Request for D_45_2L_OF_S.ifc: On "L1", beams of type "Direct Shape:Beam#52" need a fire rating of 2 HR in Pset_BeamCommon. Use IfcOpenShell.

First a look at what the model holds.

```python
import ifcopenshell
import ifcopenshell.util.element

model = ifcopenshell.open("D_45_2L_OF_S.ifc")
print(model.schema)
storey = next(s for s in model.by_type("IfcBuildingStorey") if s.Name == "L1")
beams = [e for e in ifcopenshell.util.element.get_decomposition(storey) if e.is_a("IfcBeam")]
seen = {}
for e in beams:
    element_type = ifcopenshell.util.element.get_type(e)
    key = (element_type.Name if element_type != e and element_type else None, ifcopenshell.util.element.get_pset(e, "Pset_BeamCommon", "FireRating"))
    seen[key] = seen.get(key, 0) + 1
for (name, value), count in sorted(seen.items(), key=str):
    print(count, "x", name, "|", value)
```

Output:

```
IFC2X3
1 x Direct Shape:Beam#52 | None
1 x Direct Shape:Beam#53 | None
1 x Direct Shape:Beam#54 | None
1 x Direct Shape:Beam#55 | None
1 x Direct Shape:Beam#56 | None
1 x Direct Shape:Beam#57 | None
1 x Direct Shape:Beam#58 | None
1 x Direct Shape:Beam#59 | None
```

```python
import ifcopenshell
import ifcopenshell.api.pset
import ifcopenshell.util.element

model = ifcopenshell.open("D_45_2L_OF_S.ifc")

storey = next(s for s in model.by_type("IfcBuildingStorey") if s.Name == "L1")
beams = [e for e in ifcopenshell.util.element.get_decomposition(storey) if e.is_a("IfcBeam")]

count = 0
for e in beams:
    element_type = ifcopenshell.util.element.get_type(e)
    if element_type in (None, e) or element_type.Name != "Direct Shape:Beam#52":
        continue
    # add_pset returns the element's existing set when there is one.
    pset = ifcopenshell.api.pset.add_pset(model, product=e, name="Pset_BeamCommon")
    ifcopenshell.api.pset.edit_pset(model, pset=pset, properties={"FireRating": "2 HR"})
    count += 1

print(count, "beams updated")

model.write("D_45_2L_OF_S_edited.ifc")
```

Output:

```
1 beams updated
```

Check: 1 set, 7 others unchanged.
